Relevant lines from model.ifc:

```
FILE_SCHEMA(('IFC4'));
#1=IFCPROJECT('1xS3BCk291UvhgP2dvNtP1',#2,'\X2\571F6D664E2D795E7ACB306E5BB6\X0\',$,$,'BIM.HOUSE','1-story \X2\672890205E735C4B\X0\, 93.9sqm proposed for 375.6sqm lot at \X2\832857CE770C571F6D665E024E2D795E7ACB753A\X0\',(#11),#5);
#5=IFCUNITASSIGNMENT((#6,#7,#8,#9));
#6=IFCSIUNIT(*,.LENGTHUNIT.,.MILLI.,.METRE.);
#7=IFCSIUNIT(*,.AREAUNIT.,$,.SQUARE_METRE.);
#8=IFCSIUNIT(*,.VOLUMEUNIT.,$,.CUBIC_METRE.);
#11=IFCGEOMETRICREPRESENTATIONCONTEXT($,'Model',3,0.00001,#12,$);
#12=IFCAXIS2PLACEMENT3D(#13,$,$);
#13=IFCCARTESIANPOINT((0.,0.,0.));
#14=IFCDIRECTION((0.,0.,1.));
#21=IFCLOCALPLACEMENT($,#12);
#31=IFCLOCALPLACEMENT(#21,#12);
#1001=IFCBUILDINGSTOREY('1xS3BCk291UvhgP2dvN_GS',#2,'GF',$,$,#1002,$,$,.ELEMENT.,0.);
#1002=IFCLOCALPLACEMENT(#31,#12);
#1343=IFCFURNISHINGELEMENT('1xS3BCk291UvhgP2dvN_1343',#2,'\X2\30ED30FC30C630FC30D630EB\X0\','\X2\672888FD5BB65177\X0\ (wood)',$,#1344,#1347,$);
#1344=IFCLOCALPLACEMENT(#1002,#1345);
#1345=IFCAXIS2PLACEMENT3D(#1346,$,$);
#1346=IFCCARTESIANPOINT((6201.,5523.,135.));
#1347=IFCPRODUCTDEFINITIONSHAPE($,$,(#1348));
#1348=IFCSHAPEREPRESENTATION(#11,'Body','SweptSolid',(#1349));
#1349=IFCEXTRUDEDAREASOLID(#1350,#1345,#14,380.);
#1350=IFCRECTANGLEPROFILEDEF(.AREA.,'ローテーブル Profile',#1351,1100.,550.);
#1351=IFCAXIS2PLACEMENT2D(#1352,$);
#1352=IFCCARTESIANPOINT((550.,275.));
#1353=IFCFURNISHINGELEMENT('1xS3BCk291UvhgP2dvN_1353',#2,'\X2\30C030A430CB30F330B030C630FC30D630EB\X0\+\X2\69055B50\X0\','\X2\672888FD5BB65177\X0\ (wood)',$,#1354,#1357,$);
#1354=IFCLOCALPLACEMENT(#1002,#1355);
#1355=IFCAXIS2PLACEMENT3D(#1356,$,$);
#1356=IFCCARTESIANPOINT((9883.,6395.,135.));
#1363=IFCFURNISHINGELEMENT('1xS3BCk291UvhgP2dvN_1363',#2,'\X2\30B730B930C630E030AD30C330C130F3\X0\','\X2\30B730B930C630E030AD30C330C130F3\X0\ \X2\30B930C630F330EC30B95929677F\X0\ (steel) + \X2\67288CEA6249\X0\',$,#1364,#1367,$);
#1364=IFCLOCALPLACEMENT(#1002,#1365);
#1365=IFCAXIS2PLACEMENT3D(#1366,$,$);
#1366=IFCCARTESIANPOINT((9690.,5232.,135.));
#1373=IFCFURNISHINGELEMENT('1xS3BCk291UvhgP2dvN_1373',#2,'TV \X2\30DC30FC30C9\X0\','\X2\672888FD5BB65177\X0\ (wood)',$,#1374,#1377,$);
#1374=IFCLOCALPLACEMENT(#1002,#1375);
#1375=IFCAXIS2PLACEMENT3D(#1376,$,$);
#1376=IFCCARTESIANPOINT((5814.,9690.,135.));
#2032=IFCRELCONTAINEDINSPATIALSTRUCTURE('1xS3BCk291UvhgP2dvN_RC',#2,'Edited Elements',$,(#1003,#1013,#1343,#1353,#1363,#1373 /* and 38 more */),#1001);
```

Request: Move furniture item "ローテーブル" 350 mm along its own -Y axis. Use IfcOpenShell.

```python
import ifcopenshell
import ifcopenshell.api.geometry
import ifcopenshell.util.placement

model = ifcopenshell.open("model.ifc")

item = model.by_guid("1xS3BCk291UvhgP2dvN_1343")
matrix = ifcopenshell.util.placement.get_local_placement(item.ObjectPlacement)
matrix[:3, 3] -= matrix[:3, 1] * 350.0
ifcopenshell.api.geometry.edit_object_placement(model, product=item, matrix=matrix, is_si=False)

print(ifcopenshell.util.placement.get_local_placement(item.ObjectPlacement).round(3) + 0.0)

model.write("model_rev.ifc")
```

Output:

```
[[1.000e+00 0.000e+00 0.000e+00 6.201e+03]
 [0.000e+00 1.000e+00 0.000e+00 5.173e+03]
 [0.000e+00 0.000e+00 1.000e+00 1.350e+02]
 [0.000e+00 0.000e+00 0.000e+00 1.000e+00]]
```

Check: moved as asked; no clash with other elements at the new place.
